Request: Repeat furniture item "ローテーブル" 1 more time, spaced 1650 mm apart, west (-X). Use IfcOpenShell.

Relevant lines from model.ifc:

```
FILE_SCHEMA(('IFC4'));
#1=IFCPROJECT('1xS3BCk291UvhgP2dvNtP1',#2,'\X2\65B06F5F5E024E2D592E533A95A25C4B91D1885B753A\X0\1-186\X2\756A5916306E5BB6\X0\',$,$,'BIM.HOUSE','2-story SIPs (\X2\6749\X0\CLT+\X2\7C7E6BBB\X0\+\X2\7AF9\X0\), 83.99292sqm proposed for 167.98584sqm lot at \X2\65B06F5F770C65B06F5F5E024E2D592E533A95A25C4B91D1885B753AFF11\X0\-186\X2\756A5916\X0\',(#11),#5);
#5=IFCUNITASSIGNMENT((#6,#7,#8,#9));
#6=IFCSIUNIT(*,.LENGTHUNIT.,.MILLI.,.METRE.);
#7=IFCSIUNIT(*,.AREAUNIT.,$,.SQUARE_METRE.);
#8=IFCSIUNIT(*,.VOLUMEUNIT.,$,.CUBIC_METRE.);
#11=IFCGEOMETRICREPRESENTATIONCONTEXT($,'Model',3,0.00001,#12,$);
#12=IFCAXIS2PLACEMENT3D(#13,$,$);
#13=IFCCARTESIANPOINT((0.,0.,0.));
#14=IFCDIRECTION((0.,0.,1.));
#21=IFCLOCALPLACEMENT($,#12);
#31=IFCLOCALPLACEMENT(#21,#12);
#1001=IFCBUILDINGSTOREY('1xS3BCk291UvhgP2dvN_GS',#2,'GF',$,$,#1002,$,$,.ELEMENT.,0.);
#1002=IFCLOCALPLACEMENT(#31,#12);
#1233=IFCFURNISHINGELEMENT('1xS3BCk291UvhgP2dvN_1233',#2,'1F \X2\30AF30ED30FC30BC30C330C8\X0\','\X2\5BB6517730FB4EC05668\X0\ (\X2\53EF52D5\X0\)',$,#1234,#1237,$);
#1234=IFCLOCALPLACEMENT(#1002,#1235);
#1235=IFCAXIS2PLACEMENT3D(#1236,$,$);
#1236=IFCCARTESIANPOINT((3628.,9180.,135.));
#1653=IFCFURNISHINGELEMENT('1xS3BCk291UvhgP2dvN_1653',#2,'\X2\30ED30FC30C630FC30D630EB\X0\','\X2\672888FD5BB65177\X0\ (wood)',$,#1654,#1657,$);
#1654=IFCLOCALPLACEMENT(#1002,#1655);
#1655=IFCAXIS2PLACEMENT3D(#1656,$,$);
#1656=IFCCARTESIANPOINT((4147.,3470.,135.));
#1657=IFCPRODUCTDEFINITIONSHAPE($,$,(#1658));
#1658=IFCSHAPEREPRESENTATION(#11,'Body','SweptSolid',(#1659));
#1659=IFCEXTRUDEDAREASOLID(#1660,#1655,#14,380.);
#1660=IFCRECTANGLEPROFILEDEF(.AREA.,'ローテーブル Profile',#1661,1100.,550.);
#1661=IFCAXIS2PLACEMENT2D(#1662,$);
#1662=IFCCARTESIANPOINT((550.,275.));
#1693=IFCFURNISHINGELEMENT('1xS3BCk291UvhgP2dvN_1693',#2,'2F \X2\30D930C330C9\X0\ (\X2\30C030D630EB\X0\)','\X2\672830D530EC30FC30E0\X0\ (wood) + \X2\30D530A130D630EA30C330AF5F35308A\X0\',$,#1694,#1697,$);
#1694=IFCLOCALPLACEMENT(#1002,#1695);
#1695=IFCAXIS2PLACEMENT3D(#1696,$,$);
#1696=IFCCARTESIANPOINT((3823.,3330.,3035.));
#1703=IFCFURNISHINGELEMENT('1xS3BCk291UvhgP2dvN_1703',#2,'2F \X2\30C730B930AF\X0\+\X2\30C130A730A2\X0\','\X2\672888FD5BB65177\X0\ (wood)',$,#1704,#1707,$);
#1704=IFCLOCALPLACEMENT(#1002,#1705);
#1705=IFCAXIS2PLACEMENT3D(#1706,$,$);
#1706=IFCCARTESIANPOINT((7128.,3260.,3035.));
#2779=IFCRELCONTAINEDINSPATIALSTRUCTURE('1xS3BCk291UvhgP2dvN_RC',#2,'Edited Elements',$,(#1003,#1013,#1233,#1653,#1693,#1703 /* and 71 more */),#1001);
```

```python
import numpy as np
import ifcopenshell
import ifcopenshell.api.geometry
import ifcopenshell.api.root
import ifcopenshell.util.element
import ifcopenshell.util.placement
import ifcopenshell.util.unit

model = ifcopenshell.open("model.ifc")
unit_scale = ifcopenshell.util.unit.calculate_unit_scale(model)


def reuse_history(source, copy):
    """copy_class also copies each property set's owner history, people and application; keep the originals."""
    for rel in copy.IsDefinedBy:
        if rel.is_a("IfcRelDefinesByProperties") and (history := rel.RelatingPropertyDefinition.OwnerHistory):
            rel.RelatingPropertyDefinition.OwnerHistory = source.OwnerHistory
            ifcopenshell.util.element.remove_deep2(model, history)


source = model.by_guid("1xS3BCk291UvhgP2dvN_1653")
base = ifcopenshell.util.placement.get_local_placement(source.ObjectPlacement)
step = np.array([-1.0, 0.0, 0.0]) * 1.65 / unit_scale

for i in range(1, 2):
    copy = ifcopenshell.api.root.copy_class(model, product=source)
    copy.Representation = ifcopenshell.util.element.copy_deep(
        model, source.Representation, exclude=["IfcGeometricRepresentationContext", "IfcRepresentationMap"]
    )
    reuse_history(source, copy)
    matrix = base.copy()
    matrix[:3, 3] += i * step
    print("added at", matrix[:3, 3].round(3) + 0.0)
    ifcopenshell.api.geometry.edit_object_placement(model, product=copy, matrix=matrix, is_si=False)

model.write("model_edited.ifc")
```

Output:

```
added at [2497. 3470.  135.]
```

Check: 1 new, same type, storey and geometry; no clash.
